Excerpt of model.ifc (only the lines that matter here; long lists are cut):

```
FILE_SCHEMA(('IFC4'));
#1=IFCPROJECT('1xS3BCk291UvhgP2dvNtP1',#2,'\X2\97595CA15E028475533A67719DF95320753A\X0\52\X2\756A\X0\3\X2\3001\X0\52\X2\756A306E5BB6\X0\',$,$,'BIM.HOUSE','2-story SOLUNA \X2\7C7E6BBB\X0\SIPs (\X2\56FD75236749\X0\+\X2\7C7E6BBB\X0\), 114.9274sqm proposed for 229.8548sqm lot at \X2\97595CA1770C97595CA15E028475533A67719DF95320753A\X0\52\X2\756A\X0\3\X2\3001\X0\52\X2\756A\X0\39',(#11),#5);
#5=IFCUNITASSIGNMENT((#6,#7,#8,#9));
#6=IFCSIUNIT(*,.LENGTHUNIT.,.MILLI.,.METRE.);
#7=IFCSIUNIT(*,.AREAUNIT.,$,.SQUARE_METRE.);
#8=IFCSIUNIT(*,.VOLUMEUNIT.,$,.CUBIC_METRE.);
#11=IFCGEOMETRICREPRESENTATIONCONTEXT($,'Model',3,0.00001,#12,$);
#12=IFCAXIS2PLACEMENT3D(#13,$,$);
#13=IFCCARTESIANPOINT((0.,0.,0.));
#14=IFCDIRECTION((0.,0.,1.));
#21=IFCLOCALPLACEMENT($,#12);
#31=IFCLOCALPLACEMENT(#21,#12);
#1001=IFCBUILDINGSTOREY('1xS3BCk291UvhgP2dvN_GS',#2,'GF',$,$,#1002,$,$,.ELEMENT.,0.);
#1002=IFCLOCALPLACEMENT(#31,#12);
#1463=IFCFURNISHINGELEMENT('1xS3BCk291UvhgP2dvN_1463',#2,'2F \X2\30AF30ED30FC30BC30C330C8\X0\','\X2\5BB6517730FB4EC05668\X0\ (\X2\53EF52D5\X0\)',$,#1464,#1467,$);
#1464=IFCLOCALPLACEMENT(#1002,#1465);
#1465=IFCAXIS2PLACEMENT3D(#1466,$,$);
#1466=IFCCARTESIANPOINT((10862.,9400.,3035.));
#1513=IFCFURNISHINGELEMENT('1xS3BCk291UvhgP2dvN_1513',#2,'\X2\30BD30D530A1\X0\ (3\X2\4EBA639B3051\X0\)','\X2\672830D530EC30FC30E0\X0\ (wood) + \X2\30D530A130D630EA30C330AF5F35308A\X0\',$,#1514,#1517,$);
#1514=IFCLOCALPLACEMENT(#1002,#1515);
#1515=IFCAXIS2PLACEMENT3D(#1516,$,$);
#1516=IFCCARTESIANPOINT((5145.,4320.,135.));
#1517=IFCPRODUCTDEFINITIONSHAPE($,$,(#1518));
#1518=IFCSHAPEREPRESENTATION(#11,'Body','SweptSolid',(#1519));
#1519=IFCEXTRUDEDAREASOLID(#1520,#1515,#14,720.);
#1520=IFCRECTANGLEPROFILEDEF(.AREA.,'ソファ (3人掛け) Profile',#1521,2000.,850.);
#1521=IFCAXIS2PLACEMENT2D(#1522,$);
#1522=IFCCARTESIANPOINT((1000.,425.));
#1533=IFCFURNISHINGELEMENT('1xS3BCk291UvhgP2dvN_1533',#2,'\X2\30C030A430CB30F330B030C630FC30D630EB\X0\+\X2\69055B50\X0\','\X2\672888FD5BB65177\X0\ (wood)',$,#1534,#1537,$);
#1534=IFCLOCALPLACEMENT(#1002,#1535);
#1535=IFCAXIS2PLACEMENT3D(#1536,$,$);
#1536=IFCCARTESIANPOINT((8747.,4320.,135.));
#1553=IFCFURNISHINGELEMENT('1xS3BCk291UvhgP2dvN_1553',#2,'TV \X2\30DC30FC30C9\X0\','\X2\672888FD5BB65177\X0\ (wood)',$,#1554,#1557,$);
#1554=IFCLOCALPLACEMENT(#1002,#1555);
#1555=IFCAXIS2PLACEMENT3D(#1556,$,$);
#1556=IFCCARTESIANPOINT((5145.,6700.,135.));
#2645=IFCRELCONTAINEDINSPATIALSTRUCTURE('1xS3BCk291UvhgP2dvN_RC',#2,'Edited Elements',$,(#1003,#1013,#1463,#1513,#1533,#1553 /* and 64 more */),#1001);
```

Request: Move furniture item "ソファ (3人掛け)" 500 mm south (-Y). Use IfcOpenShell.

```python
import ifcopenshell
import ifcopenshell.api.geometry
import ifcopenshell.util.placement

model = ifcopenshell.open("model.ifc")

item = model.by_id(1513)
matrix = ifcopenshell.util.placement.get_local_placement(item.ObjectPlacement)
matrix[1, 3] -= 500.0
ifcopenshell.api.geometry.edit_object_placement(model, product=item, matrix=matrix, is_si=False)

print(ifcopenshell.util.placement.get_local_placement(item.ObjectPlacement).round(3) + 0.0)

model.write("model_v2.ifc")
```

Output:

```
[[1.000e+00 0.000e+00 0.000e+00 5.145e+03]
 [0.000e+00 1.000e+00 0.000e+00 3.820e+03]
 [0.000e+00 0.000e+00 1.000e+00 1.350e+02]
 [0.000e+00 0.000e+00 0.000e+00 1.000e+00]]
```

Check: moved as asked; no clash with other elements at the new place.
